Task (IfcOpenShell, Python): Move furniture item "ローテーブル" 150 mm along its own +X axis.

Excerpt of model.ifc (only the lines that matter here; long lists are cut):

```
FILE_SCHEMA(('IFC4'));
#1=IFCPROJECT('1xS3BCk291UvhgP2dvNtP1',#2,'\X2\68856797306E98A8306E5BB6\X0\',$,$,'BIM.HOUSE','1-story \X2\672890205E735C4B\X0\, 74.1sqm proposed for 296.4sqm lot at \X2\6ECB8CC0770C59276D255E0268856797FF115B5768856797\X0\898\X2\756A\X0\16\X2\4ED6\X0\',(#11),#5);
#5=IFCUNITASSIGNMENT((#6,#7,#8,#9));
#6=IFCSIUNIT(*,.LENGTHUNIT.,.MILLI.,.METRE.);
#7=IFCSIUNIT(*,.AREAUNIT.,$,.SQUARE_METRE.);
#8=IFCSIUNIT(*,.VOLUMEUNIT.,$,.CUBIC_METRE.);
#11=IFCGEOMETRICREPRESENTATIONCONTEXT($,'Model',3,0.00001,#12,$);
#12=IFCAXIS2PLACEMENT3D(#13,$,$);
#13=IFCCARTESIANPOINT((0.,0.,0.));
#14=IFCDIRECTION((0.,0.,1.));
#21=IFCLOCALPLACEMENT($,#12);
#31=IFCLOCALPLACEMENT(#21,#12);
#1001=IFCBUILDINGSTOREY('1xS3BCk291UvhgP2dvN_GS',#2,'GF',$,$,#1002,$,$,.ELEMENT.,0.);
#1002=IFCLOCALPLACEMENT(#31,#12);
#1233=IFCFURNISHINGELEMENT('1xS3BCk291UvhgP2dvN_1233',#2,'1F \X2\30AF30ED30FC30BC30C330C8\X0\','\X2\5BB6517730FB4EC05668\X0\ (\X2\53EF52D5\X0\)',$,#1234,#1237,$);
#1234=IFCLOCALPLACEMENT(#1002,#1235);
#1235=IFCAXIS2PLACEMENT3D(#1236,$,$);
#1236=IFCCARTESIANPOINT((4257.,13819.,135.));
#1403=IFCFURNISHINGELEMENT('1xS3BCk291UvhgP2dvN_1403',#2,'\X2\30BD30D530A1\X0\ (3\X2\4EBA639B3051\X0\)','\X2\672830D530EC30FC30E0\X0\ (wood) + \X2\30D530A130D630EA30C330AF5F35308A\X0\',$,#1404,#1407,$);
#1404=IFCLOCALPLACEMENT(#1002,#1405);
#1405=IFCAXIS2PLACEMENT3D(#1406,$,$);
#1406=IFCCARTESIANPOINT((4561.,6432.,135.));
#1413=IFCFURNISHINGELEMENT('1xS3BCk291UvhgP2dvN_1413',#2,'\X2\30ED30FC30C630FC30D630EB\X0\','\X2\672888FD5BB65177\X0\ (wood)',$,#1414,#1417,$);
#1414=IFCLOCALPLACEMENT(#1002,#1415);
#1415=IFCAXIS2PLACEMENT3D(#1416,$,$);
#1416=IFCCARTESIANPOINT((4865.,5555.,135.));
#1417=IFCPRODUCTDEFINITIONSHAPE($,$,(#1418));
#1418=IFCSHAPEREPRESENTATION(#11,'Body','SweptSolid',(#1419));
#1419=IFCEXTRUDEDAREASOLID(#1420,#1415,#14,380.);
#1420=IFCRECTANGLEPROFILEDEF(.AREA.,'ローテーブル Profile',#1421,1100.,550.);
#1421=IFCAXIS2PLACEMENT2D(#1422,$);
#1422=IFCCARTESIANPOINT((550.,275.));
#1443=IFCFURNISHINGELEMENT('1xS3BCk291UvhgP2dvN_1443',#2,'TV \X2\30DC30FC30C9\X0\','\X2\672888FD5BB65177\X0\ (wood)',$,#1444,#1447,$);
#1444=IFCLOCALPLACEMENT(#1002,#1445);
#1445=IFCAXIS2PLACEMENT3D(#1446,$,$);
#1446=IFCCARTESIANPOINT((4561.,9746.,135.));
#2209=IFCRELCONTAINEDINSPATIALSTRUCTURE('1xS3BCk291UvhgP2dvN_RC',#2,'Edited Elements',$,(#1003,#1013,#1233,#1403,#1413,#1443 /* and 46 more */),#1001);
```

```python
import ifcopenshell
import ifcopenshell.api.geometry
import ifcopenshell.util.placement

model = ifcopenshell.open("model.ifc")

item = model.by_guid("1xS3BCk291UvhgP2dvN_1413")
matrix = ifcopenshell.util.placement.get_local_placement(item.ObjectPlacement)
matrix[:3, 3] += matrix[:3, 0] * 150.0
ifcopenshell.api.geometry.edit_object_placement(model, product=item, matrix=matrix, is_si=False)

print(ifcopenshell.util.placement.get_local_placement(item.ObjectPlacement).round(3) + 0.0)

model.write("model_updated.ifc")
```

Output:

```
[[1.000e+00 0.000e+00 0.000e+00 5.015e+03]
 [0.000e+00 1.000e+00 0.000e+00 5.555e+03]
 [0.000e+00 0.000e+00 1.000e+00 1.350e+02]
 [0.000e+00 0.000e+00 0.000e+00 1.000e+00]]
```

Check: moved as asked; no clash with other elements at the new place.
